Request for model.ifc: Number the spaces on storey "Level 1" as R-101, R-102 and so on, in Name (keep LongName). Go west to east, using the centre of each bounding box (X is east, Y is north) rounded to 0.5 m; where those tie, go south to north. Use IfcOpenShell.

First a look at what the model holds.

```python
import ifcopenshell
import ifcopenshell.util.element
import ifcopenshell.util.placement

model = ifcopenshell.open("model.ifc")
print(model.schema)
storey = next(s for s in model.by_type("IfcBuildingStorey") if s.Name == "Level 1")
spaces = [e for e in ifcopenshell.util.element.get_decomposition(storey) if e.is_a("IfcSpace")]
for e in sorted(spaces, key=lambda e: e.id()):
    origin = ifcopenshell.util.placement.get_local_placement(e.ObjectPlacement)[:3, 3]
    print(e.id(), e.Name, e.LongName, origin.round(2) + 0.0, sep=" | ")
```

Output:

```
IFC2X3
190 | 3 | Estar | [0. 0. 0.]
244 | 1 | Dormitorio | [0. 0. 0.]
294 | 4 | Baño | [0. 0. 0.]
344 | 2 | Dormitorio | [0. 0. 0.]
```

```python
import ifcopenshell
import ifcopenshell.geom
import ifcopenshell.util.element
import ifcopenshell.util.shape

model = ifcopenshell.open("model.ifc")
settings = ifcopenshell.geom.settings()
settings.set("use-world-coords", True)


def centre(element):
    shape = ifcopenshell.geom.create_shape(settings, element)
    return ifcopenshell.util.shape.get_bbox_centroid(shape.geometry)


storey = next(s for s in model.by_type("IfcBuildingStorey") if s.Name == "Level 1")
spaces = [e for e in ifcopenshell.util.element.get_decomposition(storey) if e.is_a("IfcSpace")]

# Insertion points can sit at a corner or the storey origin, so sort by the geometry (in metres).
centres = {e: centre(e) for e in spaces}
spaces.sort(key=lambda e: (round(centres[e][0] / 0.5), centres[e][1]))

for i, e in enumerate(spaces, start=1):
    number = f"R-1{i:02d}"
    e.Name = number
    print(e.id(), number)

model.write("model_edited.ifc")
```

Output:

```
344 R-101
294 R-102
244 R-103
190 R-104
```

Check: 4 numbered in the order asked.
